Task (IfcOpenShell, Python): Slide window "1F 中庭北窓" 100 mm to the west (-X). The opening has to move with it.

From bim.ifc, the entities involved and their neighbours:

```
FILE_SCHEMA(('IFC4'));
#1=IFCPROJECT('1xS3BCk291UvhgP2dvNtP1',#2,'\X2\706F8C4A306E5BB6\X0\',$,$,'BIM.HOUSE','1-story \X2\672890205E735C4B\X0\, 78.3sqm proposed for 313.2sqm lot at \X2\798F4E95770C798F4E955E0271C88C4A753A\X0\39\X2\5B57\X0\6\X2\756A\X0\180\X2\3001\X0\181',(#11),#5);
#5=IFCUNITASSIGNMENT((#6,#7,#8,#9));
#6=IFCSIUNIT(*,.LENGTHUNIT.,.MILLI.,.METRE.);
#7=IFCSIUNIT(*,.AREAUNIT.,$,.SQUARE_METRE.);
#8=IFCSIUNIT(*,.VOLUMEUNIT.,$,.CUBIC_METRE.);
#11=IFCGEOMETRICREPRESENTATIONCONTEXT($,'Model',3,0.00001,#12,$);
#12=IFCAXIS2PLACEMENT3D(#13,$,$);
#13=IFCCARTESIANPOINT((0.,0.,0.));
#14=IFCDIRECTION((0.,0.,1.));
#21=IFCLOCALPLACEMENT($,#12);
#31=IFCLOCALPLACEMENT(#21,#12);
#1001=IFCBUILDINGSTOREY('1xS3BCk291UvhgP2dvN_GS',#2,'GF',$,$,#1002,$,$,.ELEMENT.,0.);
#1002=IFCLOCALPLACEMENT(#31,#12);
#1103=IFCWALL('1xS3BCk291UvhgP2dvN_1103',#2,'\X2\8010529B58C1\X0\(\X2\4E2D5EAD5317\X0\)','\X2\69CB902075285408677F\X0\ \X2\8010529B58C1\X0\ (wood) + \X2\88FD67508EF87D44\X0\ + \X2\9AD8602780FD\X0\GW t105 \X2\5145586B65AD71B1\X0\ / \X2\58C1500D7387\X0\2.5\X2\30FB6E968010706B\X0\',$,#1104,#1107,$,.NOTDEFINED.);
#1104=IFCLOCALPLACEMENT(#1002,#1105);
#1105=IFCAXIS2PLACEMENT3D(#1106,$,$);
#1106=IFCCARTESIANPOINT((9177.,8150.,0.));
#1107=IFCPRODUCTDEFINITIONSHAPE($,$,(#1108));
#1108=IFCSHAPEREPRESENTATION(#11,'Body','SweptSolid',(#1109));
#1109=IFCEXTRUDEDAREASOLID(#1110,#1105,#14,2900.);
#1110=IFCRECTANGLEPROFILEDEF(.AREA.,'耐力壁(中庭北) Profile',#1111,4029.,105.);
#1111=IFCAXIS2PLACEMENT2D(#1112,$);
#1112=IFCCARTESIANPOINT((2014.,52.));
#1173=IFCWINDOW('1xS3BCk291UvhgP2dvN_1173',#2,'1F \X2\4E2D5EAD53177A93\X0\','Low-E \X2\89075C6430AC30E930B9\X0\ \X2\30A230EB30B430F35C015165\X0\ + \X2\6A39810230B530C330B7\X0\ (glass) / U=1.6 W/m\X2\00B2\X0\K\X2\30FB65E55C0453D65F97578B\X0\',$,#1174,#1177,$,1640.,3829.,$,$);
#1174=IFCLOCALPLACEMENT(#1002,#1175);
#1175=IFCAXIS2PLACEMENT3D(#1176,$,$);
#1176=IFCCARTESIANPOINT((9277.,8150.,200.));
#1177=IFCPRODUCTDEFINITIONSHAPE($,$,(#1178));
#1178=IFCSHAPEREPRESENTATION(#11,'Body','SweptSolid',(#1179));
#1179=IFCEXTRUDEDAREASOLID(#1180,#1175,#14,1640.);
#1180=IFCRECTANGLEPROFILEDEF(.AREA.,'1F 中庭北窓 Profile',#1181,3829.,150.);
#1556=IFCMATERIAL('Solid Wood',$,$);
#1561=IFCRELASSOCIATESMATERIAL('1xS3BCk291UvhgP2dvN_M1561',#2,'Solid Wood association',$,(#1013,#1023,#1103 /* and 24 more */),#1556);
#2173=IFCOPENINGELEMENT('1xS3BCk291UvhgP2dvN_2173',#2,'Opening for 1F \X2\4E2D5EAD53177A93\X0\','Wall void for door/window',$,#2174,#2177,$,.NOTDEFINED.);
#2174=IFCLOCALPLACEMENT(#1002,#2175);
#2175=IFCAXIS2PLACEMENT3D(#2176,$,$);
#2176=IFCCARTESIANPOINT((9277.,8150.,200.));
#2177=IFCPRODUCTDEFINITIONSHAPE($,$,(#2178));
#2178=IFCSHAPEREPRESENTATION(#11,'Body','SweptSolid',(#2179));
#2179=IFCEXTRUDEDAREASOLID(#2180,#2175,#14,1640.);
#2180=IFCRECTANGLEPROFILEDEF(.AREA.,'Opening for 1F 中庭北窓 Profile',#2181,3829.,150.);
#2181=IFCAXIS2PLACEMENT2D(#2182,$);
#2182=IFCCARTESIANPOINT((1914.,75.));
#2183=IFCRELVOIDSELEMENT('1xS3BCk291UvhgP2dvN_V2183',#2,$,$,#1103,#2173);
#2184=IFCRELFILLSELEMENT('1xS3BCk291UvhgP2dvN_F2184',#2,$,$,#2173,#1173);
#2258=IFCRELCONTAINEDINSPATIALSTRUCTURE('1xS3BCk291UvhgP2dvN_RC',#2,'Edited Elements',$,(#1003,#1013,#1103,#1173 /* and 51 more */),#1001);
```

```python
import ifcopenshell
import ifcopenshell.api.geometry
import ifcopenshell.util.placement

model = ifcopenshell.open("bim.ifc")

window = model.by_guid("1xS3BCk291UvhgP2dvN_1173")
opening = window.FillsVoids[0].RelatingOpeningElement
wall = opening.VoidsElements[0].RelatingBuildingElement

wall_matrix = ifcopenshell.util.placement.get_local_placement(wall.ObjectPlacement)
shift = wall_matrix[:3, 0] * -100.0
before = ifcopenshell.util.placement.get_local_placement(window.ObjectPlacement)[:3, 3].copy()

# The window is not placed relative to its opening, so move both.
for product in (opening, window):
    matrix = ifcopenshell.util.placement.get_local_placement(product.ObjectPlacement)
    matrix[:3, 3] += shift
    ifcopenshell.api.geometry.edit_object_placement(model, product=product, matrix=matrix, is_si=False)

after = ifcopenshell.util.placement.get_local_placement(window.ObjectPlacement)[:3, 3]
print("window moved by", (after - before).round(3) + 0.0)

model.write("bim_rev.ifc")
```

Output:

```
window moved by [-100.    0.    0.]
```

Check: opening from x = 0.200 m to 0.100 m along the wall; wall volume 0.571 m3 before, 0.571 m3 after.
